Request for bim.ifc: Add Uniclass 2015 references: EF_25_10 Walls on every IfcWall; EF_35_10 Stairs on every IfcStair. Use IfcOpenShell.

First a look at what the model holds.

```python
import ifcopenshell

model = ifcopenshell.open("bim.ifc")
print(model.schema)
print("classifications:", [c.Name for c in model.by_type("IfcClassification")])
for ifc_class in ("IfcDoor", "IfcRoof", "IfcStair", "IfcWall", "IfcWindow"):
    print(ifc_class, len(model.by_type(ifc_class)))
```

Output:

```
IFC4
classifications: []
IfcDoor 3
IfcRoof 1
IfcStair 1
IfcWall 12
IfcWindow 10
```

```python
import ifcopenshell
import ifcopenshell.api.classification

model = ifcopenshell.open("bim.ifc")

system = ifcopenshell.api.classification.add_classification(model, classification="Uniclass 2015")

codes = {
    "IfcWall": ("EF_25_10", "Walls"),
    "IfcStair": ("EF_35_10", "Stairs"),
}
for ifc_class, (code, name) in codes.items():
    products = model.by_type(ifc_class)
    ifcopenshell.api.classification.add_reference(
        model, products=products, classification=system, identification=code, name=name
    )
    print(code, len(products))

model.write("bim_rev.ifc")
```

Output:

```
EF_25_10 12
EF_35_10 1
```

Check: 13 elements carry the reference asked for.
